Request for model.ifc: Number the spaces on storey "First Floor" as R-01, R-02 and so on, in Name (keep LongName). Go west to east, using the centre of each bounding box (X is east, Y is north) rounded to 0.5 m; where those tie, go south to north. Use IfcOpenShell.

First a look at what the model holds.

```python
import ifcopenshell
import ifcopenshell.util.element
import ifcopenshell.util.placement

model = ifcopenshell.open("model.ifc")
print(model.schema)
storey = next(s for s in model.by_type("IfcBuildingStorey") if s.Name == "First Floor")
spaces = [e for e in ifcopenshell.util.element.get_decomposition(storey) if e.is_a("IfcSpace")]
for e in sorted(spaces, key=lambda e: e.id()):
    origin = ifcopenshell.util.placement.get_local_placement(e.ObjectPlacement)[:3, 3]
    print(e.id(), e.Name, e.LongName, origin.round(2) + 0.0, sep=" | ")
```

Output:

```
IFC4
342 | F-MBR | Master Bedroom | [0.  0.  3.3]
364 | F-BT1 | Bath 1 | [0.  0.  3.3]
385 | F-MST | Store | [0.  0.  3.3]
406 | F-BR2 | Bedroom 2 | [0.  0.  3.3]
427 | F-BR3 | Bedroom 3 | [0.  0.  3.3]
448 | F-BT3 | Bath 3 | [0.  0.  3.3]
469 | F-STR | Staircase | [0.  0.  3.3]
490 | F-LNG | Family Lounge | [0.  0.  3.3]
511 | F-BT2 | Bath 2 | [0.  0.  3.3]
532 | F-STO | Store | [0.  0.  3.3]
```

```python
import ifcopenshell
import ifcopenshell.geom
import ifcopenshell.util.element
import ifcopenshell.util.shape

model = ifcopenshell.open("model.ifc")
settings = ifcopenshell.geom.settings()
settings.set("use-world-coords", True)


def centre(element):
    shape = ifcopenshell.geom.create_shape(settings, element)
    return ifcopenshell.util.shape.get_bbox_centroid(shape.geometry)


storey = next(s for s in model.by_type("IfcBuildingStorey") if s.Name == "First Floor")
spaces = [e for e in ifcopenshell.util.element.get_decomposition(storey) if e.is_a("IfcSpace")]

# Insertion points can sit at a corner or the storey origin, so sort by the geometry (in metres).
centres = {e: centre(e) for e in spaces}
spaces.sort(key=lambda e: (round(centres[e][0] / 0.5), centres[e][1]))

for i, e in enumerate(spaces, start=1):
    number = f"R-{i:02d}"
    e.Name = number
    print(e.id(), number)

model.write("model_v2.ifc")
```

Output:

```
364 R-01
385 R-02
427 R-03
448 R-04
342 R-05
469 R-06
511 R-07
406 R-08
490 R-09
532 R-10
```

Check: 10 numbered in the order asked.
